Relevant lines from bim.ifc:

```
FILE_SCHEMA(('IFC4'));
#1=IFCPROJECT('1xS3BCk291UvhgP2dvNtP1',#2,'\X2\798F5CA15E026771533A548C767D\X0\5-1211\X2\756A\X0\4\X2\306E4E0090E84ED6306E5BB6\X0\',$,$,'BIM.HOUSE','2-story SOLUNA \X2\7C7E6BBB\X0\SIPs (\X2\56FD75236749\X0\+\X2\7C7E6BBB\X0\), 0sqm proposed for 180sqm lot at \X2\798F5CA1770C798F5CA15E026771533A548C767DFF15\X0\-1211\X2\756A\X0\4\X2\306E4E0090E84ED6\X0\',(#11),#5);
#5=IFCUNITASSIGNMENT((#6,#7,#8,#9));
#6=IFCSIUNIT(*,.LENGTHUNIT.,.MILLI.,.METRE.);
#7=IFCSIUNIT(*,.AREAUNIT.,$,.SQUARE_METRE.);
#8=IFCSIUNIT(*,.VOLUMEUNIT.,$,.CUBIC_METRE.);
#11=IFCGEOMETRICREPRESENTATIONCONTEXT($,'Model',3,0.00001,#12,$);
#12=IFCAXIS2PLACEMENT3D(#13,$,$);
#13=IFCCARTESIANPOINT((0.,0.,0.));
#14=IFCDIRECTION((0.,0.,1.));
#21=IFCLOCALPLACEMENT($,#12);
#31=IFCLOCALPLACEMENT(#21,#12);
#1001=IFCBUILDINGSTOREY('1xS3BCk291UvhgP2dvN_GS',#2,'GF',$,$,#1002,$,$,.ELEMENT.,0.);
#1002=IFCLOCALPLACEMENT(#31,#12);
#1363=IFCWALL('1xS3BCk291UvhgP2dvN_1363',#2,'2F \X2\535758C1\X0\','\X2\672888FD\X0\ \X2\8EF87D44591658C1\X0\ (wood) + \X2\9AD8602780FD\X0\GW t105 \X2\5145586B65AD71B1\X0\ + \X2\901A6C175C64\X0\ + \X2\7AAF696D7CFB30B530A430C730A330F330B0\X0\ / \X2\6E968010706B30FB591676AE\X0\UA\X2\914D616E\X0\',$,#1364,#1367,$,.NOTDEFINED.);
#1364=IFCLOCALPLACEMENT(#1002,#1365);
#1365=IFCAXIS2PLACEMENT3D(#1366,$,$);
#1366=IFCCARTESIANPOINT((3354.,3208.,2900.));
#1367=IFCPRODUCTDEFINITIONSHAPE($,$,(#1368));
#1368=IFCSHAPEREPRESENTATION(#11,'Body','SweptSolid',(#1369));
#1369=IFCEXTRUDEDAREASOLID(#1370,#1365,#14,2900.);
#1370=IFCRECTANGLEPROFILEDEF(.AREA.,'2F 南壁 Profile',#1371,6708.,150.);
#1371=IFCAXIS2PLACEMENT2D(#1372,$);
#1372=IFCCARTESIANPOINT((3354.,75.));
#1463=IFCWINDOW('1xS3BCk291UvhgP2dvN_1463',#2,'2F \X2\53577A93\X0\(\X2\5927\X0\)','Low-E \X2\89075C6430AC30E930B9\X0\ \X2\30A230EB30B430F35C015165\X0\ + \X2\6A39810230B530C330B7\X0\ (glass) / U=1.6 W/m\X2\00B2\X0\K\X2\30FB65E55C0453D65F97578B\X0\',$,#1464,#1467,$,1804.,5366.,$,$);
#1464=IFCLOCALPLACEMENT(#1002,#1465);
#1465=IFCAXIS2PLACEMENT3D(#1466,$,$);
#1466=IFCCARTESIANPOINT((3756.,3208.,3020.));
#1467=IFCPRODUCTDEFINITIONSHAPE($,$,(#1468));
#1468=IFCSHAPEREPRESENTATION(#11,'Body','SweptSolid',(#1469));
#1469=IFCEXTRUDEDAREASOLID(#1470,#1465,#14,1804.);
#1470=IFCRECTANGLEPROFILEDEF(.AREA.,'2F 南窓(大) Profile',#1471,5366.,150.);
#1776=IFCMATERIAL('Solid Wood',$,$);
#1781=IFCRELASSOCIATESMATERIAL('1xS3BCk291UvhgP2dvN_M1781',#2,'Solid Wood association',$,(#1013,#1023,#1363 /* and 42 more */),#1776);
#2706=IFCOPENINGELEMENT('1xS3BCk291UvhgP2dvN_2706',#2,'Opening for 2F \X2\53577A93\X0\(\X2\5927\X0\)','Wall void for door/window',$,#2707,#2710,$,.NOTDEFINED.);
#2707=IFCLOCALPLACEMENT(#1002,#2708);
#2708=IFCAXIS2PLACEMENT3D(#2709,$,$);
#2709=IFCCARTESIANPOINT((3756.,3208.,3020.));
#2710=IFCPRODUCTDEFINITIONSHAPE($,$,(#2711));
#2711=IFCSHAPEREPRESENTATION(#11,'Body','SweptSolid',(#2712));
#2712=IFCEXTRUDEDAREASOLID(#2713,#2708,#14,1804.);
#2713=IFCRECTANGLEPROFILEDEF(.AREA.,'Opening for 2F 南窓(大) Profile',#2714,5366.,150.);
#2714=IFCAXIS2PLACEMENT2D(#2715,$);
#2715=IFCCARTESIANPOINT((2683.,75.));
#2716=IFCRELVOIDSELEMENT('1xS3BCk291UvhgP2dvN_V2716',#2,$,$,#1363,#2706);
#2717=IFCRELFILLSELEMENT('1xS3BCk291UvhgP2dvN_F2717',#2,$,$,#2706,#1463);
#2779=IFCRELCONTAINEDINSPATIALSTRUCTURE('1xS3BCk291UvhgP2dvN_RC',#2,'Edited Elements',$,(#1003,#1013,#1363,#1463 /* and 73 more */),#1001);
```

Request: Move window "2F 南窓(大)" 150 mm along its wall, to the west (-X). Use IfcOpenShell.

```python
import ifcopenshell
import ifcopenshell.api.geometry
import ifcopenshell.util.placement
import ifcopenshell.util.unit

model = ifcopenshell.open("bim.ifc")
unit_scale = ifcopenshell.util.unit.calculate_unit_scale(model)

window = model.by_id(1463)
opening = window.FillsVoids[0].RelatingOpeningElement
wall = opening.VoidsElements[0].RelatingBuildingElement

wall_matrix = ifcopenshell.util.placement.get_local_placement(wall.ObjectPlacement)
shift = wall_matrix[:3, 0] * -0.15 / unit_scale
before = ifcopenshell.util.placement.get_local_placement(window.ObjectPlacement)[:3, 3].copy()

# The window is not placed relative to its opening, so move both.
for product in (opening, window):
    matrix = ifcopenshell.util.placement.get_local_placement(product.ObjectPlacement)
    matrix[:3, 3] += shift
    ifcopenshell.api.geometry.edit_object_placement(model, product=product, matrix=matrix, is_si=False)

after = ifcopenshell.util.placement.get_local_placement(window.ObjectPlacement)[:3, 3]
print("window moved by", (after - before).round(3) + 0.0)

model.write("bim_rev.ifc")
```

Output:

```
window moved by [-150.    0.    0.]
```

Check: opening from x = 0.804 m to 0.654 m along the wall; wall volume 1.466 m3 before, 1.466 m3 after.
